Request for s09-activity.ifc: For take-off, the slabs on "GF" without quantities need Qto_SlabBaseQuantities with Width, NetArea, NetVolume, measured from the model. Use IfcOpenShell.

First a look at what the model holds.

```python
import ifcopenshell
import ifcopenshell.util.element
import ifcopenshell.util.unit

model = ifcopenshell.open("s09-activity.ifc")
print(model.schema)
for unit_type in ("LENGTHUNIT", "AREAUNIT", "VOLUMEUNIT"):
    print(unit_type, ifcopenshell.util.unit.calculate_unit_scale(model, unit_type))
storey = next(s for s in model.by_type("IfcBuildingStorey") if s.Name == "GF")
slabs = [e for e in ifcopenshell.util.element.get_decomposition(storey) if e.is_a("IfcSlab")]
for e in sorted(slabs, key=lambda e: e.id()):
    print(e.id(), e.is_a(), e.Name, list(ifcopenshell.util.element.get_psets(e, qtos_only=True)), sep=" | ")
```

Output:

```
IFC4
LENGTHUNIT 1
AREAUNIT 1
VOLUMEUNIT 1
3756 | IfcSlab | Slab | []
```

```python
import ifcopenshell
import ifcopenshell.api.pset
import ifcopenshell.geom
import ifcopenshell.util.element
import ifcopenshell.util.shape
import ifcopenshell.util.unit

model = ifcopenshell.open("s09-activity.ifc")
unit_scale = ifcopenshell.util.unit.calculate_unit_scale(model)
area_scale = ifcopenshell.util.unit.calculate_unit_scale(model, "AREAUNIT")
volume_scale = ifcopenshell.util.unit.calculate_unit_scale(model, "VOLUMEUNIT")
settings = ifcopenshell.geom.settings()

storey = next(s for s in model.by_type("IfcBuildingStorey") if s.Name == "GF")
slabs = [e for e in ifcopenshell.util.element.get_decomposition(storey) if e.is_a("IfcSlab")]

for e in sorted(slabs, key=lambda e: e.id()):
    if ifcopenshell.util.element.get_psets(e, qtos_only=True, should_inherit=False):
        continue
    # Geometry comes back in metres, in the element's own axes.
    shape = ifcopenshell.geom.create_shape(settings, e)
    values = {
        "Width": ifcopenshell.util.shape.get_z(shape.geometry) / unit_scale,
        "NetArea": ifcopenshell.util.shape.get_footprint_area(shape.geometry) / area_scale,
        "NetVolume": ifcopenshell.util.shape.get_volume(shape.geometry) / volume_scale,
    }
    qto = ifcopenshell.api.pset.add_qto(model, product=e, name="Qto_SlabBaseQuantities")
    ifcopenshell.api.pset.edit_qto(model, qto=qto, properties=values)
    print(e.id(), {k: round(v, 3) for k, v in values.items()})

model.write("s09-activity_edited.ifc")
```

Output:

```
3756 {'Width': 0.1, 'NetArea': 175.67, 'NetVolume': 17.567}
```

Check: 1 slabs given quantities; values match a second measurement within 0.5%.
